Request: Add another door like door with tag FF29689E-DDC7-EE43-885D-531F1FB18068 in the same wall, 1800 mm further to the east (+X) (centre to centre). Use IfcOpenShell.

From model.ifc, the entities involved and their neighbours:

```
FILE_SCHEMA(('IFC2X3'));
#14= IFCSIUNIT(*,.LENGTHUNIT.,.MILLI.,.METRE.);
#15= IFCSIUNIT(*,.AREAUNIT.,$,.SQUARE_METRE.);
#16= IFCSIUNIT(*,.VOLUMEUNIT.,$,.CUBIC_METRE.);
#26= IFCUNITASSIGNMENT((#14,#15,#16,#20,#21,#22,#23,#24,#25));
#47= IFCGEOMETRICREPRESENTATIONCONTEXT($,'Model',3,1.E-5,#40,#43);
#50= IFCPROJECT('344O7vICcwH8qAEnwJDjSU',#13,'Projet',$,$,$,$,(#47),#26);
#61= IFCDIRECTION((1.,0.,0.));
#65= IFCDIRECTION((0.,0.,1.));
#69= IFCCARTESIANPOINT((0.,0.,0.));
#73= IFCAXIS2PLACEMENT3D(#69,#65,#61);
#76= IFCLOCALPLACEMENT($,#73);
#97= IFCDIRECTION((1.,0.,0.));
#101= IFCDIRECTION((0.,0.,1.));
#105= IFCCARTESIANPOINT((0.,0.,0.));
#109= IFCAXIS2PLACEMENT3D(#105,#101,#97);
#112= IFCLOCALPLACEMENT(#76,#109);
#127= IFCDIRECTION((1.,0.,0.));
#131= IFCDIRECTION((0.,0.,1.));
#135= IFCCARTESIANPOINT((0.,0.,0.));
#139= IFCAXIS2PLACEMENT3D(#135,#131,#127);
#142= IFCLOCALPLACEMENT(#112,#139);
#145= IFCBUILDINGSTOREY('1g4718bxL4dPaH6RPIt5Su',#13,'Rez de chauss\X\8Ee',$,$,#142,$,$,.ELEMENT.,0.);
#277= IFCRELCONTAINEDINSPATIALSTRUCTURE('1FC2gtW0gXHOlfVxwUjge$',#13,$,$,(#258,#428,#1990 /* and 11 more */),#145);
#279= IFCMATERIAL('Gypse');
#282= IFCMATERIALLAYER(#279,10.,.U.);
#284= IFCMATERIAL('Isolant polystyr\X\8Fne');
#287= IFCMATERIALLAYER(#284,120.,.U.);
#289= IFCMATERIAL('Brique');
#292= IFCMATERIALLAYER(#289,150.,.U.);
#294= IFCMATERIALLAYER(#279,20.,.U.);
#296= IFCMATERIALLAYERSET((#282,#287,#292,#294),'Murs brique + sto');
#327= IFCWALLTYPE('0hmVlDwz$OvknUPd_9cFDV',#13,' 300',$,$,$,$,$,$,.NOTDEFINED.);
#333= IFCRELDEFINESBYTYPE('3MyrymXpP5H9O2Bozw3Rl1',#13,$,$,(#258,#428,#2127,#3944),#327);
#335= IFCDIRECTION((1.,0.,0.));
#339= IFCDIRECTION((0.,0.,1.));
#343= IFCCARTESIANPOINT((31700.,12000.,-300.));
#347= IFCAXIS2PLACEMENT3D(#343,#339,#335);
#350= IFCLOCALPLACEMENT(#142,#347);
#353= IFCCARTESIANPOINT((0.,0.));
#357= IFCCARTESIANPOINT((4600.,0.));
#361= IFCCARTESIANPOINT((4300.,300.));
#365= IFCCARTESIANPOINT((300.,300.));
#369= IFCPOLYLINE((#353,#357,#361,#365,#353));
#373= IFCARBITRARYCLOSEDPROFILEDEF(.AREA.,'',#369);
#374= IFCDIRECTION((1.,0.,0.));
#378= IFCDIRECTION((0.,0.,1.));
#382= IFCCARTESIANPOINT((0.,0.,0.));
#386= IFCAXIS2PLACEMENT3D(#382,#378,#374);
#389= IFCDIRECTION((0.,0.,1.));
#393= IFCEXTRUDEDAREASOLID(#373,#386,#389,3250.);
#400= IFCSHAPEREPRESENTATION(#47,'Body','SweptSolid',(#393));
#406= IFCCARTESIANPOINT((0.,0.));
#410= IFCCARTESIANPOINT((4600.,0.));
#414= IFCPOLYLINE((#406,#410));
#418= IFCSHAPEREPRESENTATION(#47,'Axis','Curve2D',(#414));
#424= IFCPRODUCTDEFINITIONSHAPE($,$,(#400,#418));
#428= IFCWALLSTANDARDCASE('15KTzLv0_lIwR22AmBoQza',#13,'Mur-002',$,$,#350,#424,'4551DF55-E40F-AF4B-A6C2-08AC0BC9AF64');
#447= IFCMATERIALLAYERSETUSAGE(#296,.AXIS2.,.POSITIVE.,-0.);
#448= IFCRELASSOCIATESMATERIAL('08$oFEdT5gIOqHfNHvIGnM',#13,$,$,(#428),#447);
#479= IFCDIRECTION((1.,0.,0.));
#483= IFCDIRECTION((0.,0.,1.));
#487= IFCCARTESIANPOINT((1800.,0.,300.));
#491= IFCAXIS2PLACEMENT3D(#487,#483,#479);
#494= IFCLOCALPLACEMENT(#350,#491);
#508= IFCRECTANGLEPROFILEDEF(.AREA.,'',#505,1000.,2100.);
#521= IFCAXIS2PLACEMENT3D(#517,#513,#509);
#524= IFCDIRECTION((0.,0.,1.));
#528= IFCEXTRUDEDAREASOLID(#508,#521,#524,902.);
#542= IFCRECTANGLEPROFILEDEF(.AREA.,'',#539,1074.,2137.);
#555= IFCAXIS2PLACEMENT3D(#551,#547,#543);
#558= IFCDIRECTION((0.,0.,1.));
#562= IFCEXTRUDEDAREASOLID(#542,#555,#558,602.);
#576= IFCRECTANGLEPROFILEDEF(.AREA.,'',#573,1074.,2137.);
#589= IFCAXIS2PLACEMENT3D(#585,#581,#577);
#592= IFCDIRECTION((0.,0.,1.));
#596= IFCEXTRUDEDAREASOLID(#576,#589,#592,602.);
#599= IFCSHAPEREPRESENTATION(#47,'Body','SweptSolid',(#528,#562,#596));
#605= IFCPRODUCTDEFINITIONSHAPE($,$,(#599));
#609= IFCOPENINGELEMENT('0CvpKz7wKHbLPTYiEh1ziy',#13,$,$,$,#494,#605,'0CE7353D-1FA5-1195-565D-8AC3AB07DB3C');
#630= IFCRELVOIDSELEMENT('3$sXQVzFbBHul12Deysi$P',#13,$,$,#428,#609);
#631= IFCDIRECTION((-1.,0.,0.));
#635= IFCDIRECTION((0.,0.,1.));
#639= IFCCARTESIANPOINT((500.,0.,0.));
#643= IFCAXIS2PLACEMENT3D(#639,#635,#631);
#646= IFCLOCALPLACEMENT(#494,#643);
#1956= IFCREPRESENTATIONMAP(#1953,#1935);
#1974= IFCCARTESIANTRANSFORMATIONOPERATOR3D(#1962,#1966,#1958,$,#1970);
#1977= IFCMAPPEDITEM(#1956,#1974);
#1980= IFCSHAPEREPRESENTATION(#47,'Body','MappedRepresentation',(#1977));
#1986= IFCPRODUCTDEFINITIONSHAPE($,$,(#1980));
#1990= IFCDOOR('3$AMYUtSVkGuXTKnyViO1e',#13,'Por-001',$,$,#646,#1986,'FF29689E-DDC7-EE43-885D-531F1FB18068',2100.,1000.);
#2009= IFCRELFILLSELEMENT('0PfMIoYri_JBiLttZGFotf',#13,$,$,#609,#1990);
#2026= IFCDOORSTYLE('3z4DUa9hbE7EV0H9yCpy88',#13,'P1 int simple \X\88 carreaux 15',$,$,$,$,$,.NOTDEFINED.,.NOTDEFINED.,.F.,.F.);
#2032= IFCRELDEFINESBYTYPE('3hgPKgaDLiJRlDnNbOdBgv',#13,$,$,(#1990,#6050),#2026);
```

```python
import ifcopenshell
import ifcopenshell.api.feature
import ifcopenshell.api.geometry
import ifcopenshell.api.root
import ifcopenshell.geom
import ifcopenshell.util.element
import ifcopenshell.util.placement
import ifcopenshell.util.shape
import ifcopenshell.util.unit

model = ifcopenshell.open("model.ifc")
unit_scale = ifcopenshell.util.unit.calculate_unit_scale(model)
settings = ifcopenshell.geom.settings()


def volume(element):
    """Net volume in cubic metres, openings subtracted."""
    shape = ifcopenshell.geom.create_shape(settings, element)
    return ifcopenshell.util.shape.get_volume(shape.geometry)


def reuse_history(source, copy):
    """copy_class also copies each property set's owner history, people and application; keep the originals."""
    for rel in copy.IsDefinedBy:
        if rel.is_a("IfcRelDefinesByProperties") and (history := rel.RelatingPropertyDefinition.OwnerHistory):
            rel.RelatingPropertyDefinition.OwnerHistory = source.OwnerHistory
            ifcopenshell.util.element.remove_deep2(model, history)


door = model.by_guid("3$AMYUtSVkGuXTKnyViO1e")
opening = door.FillsVoids[0].RelatingOpeningElement
wall = opening.VoidsElements[0].RelatingBuildingElement
before = volume(wall)
shift = ifcopenshell.util.placement.get_local_placement(wall.ObjectPlacement)[:3, 0] * 1.8 / unit_scale

# copy_class copies the void relationship, type, container and properties, but no geometry.
new_opening = ifcopenshell.api.root.copy_class(model, product=opening)
new_opening.Representation = ifcopenshell.util.element.copy_deep(
    model, opening.Representation, exclude=["IfcGeometricRepresentationContext", "IfcRepresentationMap"]
)
new_opening.Tag = None
new_door = ifcopenshell.api.root.copy_class(model, product=door)
new_door.Representation = ifcopenshell.util.element.copy_deep(
    model, door.Representation, exclude=["IfcGeometricRepresentationContext", "IfcRepresentationMap"]
)
new_door.Tag = None
reuse_history(door, new_door)
fills = ifcopenshell.api.feature.add_filling(model, opening=new_opening, element=new_door)
fills.OwnerHistory = new_door.OwnerHistory  # required in IFC2X3

for old, new in ((opening, new_opening), (door, new_door)):
    matrix = ifcopenshell.util.placement.get_local_placement(old.ObjectPlacement)
    matrix[:3, 3] += shift
    ifcopenshell.api.geometry.edit_object_placement(model, product=new, matrix=matrix, is_si=False)

after = volume(wall)

print(f"wall volume {before:.3f} -> {after:.3f} m3")

model.write("model_updated.ifc")
```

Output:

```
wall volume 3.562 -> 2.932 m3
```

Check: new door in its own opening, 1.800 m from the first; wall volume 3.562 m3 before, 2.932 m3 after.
